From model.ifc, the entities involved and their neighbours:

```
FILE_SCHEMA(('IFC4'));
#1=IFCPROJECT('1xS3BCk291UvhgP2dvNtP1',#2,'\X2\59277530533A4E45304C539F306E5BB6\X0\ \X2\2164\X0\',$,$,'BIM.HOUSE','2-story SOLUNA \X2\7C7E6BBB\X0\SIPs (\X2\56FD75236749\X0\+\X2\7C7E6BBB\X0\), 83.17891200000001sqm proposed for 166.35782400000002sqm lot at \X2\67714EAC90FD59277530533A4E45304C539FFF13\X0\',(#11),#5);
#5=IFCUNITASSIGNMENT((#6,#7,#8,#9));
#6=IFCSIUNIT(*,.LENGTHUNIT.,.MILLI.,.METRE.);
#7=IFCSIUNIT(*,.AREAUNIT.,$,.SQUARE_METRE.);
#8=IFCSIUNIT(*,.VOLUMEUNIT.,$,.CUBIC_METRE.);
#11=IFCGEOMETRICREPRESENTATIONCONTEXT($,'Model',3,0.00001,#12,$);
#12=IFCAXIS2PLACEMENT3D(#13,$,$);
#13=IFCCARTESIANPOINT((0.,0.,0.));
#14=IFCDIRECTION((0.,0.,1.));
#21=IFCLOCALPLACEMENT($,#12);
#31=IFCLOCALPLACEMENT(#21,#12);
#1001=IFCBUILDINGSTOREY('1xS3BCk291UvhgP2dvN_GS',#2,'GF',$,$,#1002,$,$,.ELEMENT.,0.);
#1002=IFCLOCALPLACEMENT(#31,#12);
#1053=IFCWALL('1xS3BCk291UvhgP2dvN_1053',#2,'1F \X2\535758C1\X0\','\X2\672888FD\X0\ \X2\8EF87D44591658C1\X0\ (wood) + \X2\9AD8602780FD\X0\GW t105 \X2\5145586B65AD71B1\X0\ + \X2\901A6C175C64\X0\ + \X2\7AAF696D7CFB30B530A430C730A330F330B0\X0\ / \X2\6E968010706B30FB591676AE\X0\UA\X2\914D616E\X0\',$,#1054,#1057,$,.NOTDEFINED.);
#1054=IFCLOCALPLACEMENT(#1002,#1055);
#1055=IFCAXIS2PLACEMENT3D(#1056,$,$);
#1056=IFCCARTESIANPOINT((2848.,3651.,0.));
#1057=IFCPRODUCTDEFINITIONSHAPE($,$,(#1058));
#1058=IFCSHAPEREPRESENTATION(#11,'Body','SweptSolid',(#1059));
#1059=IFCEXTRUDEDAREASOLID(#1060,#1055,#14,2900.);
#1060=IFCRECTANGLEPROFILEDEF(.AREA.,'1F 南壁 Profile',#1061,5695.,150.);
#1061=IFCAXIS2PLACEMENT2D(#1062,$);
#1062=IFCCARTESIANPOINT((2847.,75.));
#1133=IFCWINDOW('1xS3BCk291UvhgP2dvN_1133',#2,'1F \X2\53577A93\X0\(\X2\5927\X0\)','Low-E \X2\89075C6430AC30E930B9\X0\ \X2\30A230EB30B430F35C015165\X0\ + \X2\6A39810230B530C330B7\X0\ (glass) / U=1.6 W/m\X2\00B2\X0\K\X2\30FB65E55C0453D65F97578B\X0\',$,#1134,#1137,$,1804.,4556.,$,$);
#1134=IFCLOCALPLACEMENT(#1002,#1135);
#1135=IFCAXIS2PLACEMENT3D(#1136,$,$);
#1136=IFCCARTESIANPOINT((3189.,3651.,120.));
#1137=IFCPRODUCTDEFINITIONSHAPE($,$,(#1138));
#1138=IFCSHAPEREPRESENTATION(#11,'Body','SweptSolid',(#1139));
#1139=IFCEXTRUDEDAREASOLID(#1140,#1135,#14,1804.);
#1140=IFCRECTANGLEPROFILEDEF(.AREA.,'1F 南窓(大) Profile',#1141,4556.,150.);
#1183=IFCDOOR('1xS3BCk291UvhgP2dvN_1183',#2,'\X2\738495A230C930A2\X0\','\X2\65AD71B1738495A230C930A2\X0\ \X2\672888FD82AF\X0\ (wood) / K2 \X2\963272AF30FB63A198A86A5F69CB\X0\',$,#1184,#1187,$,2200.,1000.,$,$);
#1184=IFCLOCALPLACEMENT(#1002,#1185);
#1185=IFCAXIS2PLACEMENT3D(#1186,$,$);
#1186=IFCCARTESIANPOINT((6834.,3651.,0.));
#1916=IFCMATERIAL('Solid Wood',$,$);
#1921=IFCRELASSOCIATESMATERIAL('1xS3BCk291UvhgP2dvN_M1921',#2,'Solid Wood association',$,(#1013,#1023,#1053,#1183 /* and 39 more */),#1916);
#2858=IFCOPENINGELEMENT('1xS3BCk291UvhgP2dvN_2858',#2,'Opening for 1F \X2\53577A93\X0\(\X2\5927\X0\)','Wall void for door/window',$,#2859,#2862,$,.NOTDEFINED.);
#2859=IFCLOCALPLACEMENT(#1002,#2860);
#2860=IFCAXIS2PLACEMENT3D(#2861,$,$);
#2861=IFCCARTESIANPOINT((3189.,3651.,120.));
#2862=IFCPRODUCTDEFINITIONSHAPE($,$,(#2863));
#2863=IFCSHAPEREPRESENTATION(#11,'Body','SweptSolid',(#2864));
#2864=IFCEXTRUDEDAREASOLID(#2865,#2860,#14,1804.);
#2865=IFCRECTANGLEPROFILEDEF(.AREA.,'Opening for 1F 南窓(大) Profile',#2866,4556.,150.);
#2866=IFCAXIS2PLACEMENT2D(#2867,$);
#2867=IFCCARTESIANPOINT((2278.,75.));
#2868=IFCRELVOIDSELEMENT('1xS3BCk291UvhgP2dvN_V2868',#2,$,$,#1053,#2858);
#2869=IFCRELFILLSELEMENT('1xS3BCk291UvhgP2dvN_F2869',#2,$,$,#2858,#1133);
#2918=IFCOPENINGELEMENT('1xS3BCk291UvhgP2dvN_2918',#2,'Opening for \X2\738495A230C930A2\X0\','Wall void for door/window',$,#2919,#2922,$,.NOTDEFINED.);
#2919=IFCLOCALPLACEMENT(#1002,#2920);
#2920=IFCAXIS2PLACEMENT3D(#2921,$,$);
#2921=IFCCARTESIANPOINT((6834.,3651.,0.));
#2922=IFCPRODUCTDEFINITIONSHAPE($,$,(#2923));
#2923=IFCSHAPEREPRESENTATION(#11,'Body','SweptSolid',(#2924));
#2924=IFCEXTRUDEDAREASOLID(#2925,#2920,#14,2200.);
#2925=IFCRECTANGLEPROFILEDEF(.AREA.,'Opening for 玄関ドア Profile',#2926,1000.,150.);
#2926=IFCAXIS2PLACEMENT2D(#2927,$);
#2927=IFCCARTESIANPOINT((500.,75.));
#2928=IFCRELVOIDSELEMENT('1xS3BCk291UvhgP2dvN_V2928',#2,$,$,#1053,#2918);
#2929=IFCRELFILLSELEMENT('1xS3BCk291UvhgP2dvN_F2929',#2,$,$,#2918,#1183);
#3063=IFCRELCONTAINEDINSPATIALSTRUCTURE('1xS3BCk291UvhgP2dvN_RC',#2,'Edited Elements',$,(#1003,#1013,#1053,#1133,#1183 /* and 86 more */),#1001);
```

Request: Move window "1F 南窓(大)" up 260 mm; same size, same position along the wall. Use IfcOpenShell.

```python
import numpy as np
import ifcopenshell
import ifcopenshell.api.geometry
import ifcopenshell.util.placement
import ifcopenshell.util.unit

model = ifcopenshell.open("model.ifc")
unit_scale = ifcopenshell.util.unit.calculate_unit_scale(model)

window = model.by_guid("1xS3BCk291UvhgP2dvN_1133")
opening = window.FillsVoids[0].RelatingOpeningElement
dz = 0.26 / unit_scale

shift = np.array([0.0, 0.0, dz])
# The window is not placed relative to its opening, so move both.
for product in (opening, window):
    matrix = ifcopenshell.util.placement.get_local_placement(product.ObjectPlacement)
    matrix[:3, 3] += shift
    ifcopenshell.api.geometry.edit_object_placement(model, product=product, matrix=matrix, is_si=False)

print(f"moved by {dz * unit_scale:+.3f} m")

model.write("model_v2.ifc")
```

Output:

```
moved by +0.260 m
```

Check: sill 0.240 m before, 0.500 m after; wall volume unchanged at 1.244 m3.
